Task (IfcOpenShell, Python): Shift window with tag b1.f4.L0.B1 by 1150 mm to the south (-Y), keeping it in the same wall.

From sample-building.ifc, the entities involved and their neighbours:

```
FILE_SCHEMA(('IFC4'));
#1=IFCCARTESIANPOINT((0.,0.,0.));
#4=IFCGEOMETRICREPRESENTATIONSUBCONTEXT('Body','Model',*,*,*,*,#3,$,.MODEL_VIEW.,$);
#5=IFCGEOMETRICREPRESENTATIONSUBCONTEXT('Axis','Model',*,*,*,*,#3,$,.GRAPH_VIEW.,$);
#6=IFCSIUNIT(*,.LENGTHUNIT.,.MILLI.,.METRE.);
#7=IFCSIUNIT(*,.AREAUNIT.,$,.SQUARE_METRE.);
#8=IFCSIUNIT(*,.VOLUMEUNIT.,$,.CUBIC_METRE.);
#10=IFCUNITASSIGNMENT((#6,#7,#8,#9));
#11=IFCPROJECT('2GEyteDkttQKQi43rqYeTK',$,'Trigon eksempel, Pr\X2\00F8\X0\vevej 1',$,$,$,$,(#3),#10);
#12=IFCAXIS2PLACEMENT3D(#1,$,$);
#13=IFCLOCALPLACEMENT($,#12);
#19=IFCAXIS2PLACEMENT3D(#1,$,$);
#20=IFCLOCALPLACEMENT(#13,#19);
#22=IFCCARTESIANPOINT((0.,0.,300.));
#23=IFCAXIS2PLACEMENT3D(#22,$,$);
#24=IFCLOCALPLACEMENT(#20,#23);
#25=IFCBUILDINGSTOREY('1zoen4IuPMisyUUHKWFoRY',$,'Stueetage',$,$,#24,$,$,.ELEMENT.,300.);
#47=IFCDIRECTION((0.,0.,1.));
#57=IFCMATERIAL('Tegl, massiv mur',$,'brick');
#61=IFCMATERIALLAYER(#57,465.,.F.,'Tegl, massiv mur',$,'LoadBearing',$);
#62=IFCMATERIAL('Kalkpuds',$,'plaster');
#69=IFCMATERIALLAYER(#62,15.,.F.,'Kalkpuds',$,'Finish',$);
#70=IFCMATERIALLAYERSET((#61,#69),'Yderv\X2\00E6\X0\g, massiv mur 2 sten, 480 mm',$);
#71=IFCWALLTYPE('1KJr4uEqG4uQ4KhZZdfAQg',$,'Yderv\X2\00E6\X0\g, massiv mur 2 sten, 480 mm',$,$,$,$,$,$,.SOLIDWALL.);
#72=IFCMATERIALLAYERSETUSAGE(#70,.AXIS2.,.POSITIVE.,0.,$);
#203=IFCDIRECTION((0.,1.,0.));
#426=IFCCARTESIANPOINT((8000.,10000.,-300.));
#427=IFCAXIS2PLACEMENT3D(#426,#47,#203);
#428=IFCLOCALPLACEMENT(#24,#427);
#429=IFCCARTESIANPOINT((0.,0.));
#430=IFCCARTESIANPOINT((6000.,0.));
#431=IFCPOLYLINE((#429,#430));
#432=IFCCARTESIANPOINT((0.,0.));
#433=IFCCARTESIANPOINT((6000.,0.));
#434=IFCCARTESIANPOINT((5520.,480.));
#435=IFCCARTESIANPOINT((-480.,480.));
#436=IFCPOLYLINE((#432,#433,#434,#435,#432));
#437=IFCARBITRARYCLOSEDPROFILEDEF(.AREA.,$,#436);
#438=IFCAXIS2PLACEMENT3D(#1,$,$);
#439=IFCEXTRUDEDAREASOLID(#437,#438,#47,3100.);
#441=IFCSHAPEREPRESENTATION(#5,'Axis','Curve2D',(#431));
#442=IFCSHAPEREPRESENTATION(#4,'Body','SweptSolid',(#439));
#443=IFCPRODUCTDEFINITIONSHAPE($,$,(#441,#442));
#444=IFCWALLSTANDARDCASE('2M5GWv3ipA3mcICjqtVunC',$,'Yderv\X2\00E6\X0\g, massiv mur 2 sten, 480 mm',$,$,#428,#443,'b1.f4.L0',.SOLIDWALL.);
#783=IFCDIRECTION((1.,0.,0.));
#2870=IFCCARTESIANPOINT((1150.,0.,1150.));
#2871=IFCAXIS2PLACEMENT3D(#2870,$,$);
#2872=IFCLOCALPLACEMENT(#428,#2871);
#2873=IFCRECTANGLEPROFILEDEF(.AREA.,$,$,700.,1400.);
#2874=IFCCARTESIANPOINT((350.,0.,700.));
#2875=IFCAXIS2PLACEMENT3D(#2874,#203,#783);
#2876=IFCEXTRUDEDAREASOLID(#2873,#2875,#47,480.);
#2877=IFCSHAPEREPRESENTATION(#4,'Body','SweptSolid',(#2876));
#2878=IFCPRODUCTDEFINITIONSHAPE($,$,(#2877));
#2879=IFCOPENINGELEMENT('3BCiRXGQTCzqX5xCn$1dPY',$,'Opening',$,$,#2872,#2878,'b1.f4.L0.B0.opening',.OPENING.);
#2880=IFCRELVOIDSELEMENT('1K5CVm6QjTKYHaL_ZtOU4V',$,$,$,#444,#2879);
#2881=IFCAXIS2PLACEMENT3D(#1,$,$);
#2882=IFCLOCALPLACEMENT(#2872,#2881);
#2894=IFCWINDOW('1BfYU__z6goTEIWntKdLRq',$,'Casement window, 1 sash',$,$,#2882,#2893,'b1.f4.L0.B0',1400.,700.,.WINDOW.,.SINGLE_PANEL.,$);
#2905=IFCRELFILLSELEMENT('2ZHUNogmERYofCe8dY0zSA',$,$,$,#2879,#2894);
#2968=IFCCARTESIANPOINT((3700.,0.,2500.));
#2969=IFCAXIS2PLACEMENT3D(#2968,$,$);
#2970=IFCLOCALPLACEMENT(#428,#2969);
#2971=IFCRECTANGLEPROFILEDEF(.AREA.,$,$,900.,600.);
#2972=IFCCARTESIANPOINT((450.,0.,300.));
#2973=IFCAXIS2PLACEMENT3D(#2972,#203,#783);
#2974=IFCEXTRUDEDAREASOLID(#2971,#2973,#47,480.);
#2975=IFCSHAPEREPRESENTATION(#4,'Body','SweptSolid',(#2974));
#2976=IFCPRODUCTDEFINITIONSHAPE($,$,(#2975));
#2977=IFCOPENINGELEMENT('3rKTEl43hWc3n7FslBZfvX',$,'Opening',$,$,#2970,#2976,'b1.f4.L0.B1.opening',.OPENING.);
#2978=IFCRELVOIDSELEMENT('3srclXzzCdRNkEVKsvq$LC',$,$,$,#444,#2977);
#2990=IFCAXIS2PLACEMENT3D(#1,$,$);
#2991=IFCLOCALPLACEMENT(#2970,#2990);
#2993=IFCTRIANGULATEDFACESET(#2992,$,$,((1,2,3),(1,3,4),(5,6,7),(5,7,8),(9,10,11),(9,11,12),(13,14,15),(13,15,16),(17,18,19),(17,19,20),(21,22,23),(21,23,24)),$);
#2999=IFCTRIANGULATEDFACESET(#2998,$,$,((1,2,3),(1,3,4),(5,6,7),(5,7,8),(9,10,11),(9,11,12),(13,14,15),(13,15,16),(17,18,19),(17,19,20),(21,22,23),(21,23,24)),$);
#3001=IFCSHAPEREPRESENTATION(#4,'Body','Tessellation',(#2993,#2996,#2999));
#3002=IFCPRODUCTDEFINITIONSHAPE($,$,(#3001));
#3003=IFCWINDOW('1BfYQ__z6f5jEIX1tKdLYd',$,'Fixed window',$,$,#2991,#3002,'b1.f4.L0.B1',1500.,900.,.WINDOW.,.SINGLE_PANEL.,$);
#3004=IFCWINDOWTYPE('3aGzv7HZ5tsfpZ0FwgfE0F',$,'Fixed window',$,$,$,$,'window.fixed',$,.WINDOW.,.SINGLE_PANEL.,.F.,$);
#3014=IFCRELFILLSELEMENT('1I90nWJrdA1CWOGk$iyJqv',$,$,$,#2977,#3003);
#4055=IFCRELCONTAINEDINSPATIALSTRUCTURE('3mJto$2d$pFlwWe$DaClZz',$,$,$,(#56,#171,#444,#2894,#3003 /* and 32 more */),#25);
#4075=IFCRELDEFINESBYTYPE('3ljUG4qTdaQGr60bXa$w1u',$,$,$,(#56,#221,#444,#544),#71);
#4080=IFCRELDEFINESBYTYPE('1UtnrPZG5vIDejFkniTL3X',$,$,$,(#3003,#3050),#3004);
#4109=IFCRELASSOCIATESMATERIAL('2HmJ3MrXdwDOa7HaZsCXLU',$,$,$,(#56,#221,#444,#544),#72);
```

```python
import ifcopenshell
import ifcopenshell.api.geometry
import ifcopenshell.util.placement

model = ifcopenshell.open("sample-building.ifc")

window = model.by_guid("1BfYQ__z6f5jEIX1tKdLYd")
opening = window.FillsVoids[0].RelatingOpeningElement
wall = opening.VoidsElements[0].RelatingBuildingElement

wall_matrix = ifcopenshell.util.placement.get_local_placement(wall.ObjectPlacement)
shift = wall_matrix[:3, 0] * -1150.0
before = ifcopenshell.util.placement.get_local_placement(window.ObjectPlacement)[:3, 3].copy()

# The window is placed relative to its opening, so it follows when the opening moves.
matrix = ifcopenshell.util.placement.get_local_placement(opening.ObjectPlacement)
matrix[:3, 3] += shift
ifcopenshell.api.geometry.edit_object_placement(
    model, product=opening, matrix=matrix, is_si=False, should_transform_children=True
)

after = ifcopenshell.util.placement.get_local_placement(window.ObjectPlacement)[:3, 3]
print("window moved by", (after - before).round(3) + 0.0)

model.write("sample-building_updated.ifc")
```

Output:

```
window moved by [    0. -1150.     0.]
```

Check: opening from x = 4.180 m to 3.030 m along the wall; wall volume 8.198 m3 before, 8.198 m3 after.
